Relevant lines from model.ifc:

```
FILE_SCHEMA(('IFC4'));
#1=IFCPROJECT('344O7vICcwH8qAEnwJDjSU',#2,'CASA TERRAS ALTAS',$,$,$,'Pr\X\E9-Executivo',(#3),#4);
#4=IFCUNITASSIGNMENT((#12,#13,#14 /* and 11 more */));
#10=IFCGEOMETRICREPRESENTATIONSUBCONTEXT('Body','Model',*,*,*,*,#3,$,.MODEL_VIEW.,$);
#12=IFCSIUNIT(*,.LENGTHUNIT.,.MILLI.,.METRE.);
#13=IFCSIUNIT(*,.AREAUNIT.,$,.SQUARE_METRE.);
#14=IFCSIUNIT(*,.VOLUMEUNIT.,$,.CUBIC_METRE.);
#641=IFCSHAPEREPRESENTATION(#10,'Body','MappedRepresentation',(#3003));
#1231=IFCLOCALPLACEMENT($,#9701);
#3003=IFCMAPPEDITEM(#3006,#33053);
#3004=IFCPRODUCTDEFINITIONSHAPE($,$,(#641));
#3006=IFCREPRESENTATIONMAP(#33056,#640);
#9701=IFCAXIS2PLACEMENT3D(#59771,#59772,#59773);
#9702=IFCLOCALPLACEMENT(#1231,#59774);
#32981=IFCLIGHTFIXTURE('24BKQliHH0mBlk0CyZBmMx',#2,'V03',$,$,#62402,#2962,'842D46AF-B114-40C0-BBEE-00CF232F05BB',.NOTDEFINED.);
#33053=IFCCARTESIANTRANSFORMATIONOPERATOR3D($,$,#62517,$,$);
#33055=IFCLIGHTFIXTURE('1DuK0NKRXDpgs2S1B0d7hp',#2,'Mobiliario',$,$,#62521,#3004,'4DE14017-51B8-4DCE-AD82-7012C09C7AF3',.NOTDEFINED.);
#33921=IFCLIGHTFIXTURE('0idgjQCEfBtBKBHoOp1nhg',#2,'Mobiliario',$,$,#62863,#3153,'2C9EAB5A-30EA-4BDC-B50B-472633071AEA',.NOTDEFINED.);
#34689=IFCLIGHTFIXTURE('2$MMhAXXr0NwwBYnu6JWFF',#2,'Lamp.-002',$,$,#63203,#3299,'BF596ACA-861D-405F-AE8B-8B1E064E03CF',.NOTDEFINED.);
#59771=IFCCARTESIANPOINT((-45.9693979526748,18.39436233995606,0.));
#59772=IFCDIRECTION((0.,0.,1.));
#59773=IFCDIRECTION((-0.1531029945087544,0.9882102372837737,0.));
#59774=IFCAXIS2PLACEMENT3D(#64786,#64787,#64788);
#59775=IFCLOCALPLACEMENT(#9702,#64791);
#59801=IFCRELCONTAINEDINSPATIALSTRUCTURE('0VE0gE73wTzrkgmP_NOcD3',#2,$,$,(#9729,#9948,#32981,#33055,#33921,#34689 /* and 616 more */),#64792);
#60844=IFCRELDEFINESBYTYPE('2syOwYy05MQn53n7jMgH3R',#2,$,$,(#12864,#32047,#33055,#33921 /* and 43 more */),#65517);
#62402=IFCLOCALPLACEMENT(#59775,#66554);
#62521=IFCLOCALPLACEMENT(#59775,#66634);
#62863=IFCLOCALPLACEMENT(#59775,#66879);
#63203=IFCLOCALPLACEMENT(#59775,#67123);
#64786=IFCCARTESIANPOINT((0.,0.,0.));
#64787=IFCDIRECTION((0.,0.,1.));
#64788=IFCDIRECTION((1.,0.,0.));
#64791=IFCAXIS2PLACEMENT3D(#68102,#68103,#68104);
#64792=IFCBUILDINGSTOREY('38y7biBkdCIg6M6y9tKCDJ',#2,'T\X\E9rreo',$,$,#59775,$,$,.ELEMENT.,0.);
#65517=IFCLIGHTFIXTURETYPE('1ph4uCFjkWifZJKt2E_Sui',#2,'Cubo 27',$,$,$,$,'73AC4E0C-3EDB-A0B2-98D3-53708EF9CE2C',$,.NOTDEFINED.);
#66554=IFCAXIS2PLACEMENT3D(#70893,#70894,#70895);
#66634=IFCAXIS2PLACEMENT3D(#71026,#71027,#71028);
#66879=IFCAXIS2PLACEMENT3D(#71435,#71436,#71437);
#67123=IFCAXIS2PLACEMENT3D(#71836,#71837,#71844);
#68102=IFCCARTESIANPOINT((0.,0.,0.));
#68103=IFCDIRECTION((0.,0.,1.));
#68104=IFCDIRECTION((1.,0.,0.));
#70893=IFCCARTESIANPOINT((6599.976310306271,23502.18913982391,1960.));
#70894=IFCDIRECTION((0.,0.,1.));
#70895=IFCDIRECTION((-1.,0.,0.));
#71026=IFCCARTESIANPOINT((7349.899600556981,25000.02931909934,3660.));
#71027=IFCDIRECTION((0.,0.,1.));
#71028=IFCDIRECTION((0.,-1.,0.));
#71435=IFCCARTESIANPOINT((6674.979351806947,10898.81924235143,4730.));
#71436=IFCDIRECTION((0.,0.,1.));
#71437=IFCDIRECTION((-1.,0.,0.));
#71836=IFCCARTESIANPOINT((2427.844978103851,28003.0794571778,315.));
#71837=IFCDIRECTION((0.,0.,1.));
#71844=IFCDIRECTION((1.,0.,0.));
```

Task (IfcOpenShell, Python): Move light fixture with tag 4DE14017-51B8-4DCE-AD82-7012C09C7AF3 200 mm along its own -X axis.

```python
import ifcopenshell
import ifcopenshell.api.geometry
import ifcopenshell.util.placement

model = ifcopenshell.open("model.ifc")

item = model.by_guid("1DuK0NKRXDpgs2S1B0d7hp")
matrix = ifcopenshell.util.placement.get_local_placement(item.ObjectPlacement)
matrix[:3, 3] -= matrix[:3, 0] * 200.0
ifcopenshell.api.geometry.edit_object_placement(model, product=item, matrix=matrix, is_si=False)

print(ifcopenshell.util.placement.get_local_placement(item.ObjectPlacement).round(3) + 0.0)

model.write("model_edited.ifc")
```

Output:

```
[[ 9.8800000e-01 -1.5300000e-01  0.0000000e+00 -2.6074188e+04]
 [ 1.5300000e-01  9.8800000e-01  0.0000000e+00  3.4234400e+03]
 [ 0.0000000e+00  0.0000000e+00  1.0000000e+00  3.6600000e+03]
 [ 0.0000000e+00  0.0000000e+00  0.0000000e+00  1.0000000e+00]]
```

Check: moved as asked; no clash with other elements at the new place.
